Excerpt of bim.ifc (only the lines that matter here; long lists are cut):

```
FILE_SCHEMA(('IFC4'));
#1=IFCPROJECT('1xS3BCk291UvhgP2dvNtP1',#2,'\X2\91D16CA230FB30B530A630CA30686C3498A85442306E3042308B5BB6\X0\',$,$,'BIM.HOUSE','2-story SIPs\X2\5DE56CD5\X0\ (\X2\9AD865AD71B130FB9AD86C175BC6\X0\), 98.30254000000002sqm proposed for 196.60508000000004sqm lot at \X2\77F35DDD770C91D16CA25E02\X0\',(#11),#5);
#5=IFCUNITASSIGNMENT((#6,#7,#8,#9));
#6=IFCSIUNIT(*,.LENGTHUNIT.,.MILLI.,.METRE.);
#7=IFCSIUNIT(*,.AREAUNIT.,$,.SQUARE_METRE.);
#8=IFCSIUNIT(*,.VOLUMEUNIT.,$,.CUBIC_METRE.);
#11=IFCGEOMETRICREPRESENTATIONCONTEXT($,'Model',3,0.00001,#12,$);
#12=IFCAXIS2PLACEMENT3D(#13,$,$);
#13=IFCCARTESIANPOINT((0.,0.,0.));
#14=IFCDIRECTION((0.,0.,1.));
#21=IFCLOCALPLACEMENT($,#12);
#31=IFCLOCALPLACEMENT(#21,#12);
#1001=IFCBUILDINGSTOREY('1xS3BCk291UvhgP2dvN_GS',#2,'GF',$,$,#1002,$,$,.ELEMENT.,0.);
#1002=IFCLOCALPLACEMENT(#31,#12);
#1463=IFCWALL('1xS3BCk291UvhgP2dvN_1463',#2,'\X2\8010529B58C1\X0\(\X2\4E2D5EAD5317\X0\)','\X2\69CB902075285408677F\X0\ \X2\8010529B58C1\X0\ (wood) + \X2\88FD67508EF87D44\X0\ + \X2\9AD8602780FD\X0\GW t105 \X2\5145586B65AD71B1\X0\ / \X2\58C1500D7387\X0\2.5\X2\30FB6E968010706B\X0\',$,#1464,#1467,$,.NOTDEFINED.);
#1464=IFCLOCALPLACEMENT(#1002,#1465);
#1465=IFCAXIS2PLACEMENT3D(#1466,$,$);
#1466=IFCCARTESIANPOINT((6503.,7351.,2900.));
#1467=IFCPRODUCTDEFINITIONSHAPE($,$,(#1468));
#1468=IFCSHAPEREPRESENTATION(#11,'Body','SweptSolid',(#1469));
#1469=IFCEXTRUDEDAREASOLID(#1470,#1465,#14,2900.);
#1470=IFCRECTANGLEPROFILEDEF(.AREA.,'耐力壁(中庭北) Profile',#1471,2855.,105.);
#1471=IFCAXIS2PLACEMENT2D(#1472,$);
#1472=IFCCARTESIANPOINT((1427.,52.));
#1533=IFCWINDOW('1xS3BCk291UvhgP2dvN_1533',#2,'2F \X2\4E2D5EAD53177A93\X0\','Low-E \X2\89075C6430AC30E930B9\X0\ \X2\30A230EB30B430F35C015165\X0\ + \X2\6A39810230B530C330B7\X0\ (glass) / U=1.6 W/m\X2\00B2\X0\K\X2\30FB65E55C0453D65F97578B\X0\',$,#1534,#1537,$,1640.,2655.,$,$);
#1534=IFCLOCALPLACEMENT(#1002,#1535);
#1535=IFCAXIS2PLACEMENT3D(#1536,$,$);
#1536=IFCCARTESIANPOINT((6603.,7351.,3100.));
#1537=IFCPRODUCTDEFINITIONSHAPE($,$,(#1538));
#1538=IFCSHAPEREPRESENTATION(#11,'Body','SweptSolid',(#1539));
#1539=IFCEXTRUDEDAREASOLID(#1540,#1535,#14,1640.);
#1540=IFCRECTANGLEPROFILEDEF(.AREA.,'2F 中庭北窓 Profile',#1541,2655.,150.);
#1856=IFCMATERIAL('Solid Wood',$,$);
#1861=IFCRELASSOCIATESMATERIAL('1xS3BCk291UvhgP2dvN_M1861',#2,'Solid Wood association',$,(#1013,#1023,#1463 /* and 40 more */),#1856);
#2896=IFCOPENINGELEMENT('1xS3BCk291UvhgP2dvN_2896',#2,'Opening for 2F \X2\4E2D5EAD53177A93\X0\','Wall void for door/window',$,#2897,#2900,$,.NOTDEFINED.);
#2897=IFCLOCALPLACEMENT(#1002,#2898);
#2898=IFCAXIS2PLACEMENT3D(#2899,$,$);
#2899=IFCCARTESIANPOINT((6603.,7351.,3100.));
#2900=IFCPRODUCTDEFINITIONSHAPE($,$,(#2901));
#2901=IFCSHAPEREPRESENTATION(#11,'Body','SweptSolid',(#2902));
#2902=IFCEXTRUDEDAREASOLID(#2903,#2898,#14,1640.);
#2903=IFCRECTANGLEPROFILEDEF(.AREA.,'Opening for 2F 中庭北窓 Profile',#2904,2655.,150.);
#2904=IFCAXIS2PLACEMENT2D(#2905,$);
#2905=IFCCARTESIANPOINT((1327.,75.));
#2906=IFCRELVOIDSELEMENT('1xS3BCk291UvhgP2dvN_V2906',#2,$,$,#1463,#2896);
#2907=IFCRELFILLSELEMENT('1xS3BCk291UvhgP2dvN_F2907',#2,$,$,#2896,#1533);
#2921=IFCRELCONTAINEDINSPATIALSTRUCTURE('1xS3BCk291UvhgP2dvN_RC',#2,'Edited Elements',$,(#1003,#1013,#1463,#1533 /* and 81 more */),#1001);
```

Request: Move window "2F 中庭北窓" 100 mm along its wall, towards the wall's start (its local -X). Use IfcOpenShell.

```python
import ifcopenshell
import ifcopenshell.api.geometry
import ifcopenshell.util.placement
import ifcopenshell.util.unit

model = ifcopenshell.open("bim.ifc")
unit_scale = ifcopenshell.util.unit.calculate_unit_scale(model)

window = model.by_id(1533)
opening = window.FillsVoids[0].RelatingOpeningElement
wall = opening.VoidsElements[0].RelatingBuildingElement

wall_matrix = ifcopenshell.util.placement.get_local_placement(wall.ObjectPlacement)
shift = wall_matrix[:3, 0] * -0.1 / unit_scale
before = ifcopenshell.util.placement.get_local_placement(window.ObjectPlacement)[:3, 3].copy()

# The window is not placed relative to its opening, so move both.
for product in (opening, window):
    matrix = ifcopenshell.util.placement.get_local_placement(product.ObjectPlacement)
    matrix[:3, 3] += shift
    ifcopenshell.api.geometry.edit_object_placement(model, product=product, matrix=matrix, is_si=False)

after = ifcopenshell.util.placement.get_local_placement(window.ObjectPlacement)[:3, 3]
print("window moved by", (after - before).round(3) + 0.0)

model.write("bim_updated.ifc")
```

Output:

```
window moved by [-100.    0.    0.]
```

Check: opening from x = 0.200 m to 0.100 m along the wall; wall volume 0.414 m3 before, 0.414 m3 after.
